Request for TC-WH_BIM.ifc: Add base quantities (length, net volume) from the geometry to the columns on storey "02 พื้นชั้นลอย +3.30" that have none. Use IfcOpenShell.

First a look at what the model holds.

```python
import ifcopenshell
import ifcopenshell.util.element
import ifcopenshell.util.unit

model = ifcopenshell.open("TC-WH_BIM.ifc")
print(model.schema)
for unit_type in ("LENGTHUNIT", "AREAUNIT", "VOLUMEUNIT"):
    print(unit_type, ifcopenshell.util.unit.calculate_unit_scale(model, unit_type))
storey = next(s for s in model.by_type("IfcBuildingStorey") if s.Name == "02 พื้นชั้นลอย +3.30")
columns = [e for e in ifcopenshell.util.element.get_decomposition(storey) if e.is_a("IfcColumn")]
for e in sorted(columns, key=lambda e: e.id()):
    print(e.id(), e.is_a(), e.Name, list(ifcopenshell.util.element.get_psets(e, qtos_only=True)), sep=" | ")
```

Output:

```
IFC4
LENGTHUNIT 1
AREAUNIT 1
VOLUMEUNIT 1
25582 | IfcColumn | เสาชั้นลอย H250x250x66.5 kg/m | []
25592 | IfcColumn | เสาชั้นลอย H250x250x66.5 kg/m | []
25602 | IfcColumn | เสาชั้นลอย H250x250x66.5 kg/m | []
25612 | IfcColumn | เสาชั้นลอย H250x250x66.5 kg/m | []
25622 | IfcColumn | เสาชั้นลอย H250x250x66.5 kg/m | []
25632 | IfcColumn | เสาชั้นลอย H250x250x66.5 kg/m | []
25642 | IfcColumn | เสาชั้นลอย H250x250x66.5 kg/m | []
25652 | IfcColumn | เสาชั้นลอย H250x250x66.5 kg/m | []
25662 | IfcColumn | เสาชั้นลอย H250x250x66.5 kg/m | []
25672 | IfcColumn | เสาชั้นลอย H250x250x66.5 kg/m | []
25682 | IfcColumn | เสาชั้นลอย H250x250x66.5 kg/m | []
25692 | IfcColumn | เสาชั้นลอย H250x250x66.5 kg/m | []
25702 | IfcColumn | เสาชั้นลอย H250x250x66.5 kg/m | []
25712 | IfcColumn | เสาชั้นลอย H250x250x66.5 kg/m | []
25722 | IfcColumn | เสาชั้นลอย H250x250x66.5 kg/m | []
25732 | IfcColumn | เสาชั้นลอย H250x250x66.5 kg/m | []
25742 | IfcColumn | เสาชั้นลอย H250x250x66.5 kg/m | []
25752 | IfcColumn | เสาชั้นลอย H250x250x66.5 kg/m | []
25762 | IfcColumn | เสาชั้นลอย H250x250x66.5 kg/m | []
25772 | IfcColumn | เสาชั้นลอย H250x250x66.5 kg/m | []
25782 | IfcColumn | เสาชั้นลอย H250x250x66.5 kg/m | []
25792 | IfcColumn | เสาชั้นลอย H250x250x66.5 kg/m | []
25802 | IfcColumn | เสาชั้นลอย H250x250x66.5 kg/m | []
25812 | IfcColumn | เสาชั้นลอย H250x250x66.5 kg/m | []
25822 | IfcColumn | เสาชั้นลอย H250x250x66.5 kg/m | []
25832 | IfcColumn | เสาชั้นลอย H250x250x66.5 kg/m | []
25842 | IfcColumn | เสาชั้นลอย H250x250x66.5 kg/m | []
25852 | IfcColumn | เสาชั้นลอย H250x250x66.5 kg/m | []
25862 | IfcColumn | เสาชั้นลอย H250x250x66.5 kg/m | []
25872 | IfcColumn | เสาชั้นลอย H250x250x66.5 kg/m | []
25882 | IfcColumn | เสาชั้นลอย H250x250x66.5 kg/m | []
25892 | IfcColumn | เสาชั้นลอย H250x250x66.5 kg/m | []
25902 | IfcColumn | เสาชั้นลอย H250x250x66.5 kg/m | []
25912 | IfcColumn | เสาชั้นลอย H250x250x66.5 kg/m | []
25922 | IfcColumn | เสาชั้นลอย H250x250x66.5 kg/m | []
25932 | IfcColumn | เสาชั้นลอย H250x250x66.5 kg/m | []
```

```python
import ifcopenshell
import ifcopenshell.api.pset
import ifcopenshell.geom
import ifcopenshell.util.element
import ifcopenshell.util.shape
import ifcopenshell.util.unit

model = ifcopenshell.open("TC-WH_BIM.ifc")
unit_scale = ifcopenshell.util.unit.calculate_unit_scale(model)
volume_scale = ifcopenshell.util.unit.calculate_unit_scale(model, "VOLUMEUNIT")
settings = ifcopenshell.geom.settings()

storey = next(s for s in model.by_type("IfcBuildingStorey") if s.Name == "02 พื้นชั้นลอย +3.30")
columns = [e for e in ifcopenshell.util.element.get_decomposition(storey) if e.is_a("IfcColumn")]

for e in sorted(columns, key=lambda e: e.id()):
    if ifcopenshell.util.element.get_psets(e, qtos_only=True, should_inherit=False):
        continue
    # Geometry comes back in metres, in the element's own axes.
    shape = ifcopenshell.geom.create_shape(settings, e)
    values = {
        "Length": ifcopenshell.util.shape.get_z(shape.geometry) / unit_scale,
        "NetVolume": ifcopenshell.util.shape.get_volume(shape.geometry) / volume_scale,
    }
    qto = ifcopenshell.api.pset.add_qto(model, product=e, name="Qto_ColumnBaseQuantities")
    ifcopenshell.api.pset.edit_qto(model, qto=qto, properties=values)
    print(e.id(), {k: round(v, 3) for k, v in values.items()})

model.write("TC-WH_BIM_edited.ifc")
```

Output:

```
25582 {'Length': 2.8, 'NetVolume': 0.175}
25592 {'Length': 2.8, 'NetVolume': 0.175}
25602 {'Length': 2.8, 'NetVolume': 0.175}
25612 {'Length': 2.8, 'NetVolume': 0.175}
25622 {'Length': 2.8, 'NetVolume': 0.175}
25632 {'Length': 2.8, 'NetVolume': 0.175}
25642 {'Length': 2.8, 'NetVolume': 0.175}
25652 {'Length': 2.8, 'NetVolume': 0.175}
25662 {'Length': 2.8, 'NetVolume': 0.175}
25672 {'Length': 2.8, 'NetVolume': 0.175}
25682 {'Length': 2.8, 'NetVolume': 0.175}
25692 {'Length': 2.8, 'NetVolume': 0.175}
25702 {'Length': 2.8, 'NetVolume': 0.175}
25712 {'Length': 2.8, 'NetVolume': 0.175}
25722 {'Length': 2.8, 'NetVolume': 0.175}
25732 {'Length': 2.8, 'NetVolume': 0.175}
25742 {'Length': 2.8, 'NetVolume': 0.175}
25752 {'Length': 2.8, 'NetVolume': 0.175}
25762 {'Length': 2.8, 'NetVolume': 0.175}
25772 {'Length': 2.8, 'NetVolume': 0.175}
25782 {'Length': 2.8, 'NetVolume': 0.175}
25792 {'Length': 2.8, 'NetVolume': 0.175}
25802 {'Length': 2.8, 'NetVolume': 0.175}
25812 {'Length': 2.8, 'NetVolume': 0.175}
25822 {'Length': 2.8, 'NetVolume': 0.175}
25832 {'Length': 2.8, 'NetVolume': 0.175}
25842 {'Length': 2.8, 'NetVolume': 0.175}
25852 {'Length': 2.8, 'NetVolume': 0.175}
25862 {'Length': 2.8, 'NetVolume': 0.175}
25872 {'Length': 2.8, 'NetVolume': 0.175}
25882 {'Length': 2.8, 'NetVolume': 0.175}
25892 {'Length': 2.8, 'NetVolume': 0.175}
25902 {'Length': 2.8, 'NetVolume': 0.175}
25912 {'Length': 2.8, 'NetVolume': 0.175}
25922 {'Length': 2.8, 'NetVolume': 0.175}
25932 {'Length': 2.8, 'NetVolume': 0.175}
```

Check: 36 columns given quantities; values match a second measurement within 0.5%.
